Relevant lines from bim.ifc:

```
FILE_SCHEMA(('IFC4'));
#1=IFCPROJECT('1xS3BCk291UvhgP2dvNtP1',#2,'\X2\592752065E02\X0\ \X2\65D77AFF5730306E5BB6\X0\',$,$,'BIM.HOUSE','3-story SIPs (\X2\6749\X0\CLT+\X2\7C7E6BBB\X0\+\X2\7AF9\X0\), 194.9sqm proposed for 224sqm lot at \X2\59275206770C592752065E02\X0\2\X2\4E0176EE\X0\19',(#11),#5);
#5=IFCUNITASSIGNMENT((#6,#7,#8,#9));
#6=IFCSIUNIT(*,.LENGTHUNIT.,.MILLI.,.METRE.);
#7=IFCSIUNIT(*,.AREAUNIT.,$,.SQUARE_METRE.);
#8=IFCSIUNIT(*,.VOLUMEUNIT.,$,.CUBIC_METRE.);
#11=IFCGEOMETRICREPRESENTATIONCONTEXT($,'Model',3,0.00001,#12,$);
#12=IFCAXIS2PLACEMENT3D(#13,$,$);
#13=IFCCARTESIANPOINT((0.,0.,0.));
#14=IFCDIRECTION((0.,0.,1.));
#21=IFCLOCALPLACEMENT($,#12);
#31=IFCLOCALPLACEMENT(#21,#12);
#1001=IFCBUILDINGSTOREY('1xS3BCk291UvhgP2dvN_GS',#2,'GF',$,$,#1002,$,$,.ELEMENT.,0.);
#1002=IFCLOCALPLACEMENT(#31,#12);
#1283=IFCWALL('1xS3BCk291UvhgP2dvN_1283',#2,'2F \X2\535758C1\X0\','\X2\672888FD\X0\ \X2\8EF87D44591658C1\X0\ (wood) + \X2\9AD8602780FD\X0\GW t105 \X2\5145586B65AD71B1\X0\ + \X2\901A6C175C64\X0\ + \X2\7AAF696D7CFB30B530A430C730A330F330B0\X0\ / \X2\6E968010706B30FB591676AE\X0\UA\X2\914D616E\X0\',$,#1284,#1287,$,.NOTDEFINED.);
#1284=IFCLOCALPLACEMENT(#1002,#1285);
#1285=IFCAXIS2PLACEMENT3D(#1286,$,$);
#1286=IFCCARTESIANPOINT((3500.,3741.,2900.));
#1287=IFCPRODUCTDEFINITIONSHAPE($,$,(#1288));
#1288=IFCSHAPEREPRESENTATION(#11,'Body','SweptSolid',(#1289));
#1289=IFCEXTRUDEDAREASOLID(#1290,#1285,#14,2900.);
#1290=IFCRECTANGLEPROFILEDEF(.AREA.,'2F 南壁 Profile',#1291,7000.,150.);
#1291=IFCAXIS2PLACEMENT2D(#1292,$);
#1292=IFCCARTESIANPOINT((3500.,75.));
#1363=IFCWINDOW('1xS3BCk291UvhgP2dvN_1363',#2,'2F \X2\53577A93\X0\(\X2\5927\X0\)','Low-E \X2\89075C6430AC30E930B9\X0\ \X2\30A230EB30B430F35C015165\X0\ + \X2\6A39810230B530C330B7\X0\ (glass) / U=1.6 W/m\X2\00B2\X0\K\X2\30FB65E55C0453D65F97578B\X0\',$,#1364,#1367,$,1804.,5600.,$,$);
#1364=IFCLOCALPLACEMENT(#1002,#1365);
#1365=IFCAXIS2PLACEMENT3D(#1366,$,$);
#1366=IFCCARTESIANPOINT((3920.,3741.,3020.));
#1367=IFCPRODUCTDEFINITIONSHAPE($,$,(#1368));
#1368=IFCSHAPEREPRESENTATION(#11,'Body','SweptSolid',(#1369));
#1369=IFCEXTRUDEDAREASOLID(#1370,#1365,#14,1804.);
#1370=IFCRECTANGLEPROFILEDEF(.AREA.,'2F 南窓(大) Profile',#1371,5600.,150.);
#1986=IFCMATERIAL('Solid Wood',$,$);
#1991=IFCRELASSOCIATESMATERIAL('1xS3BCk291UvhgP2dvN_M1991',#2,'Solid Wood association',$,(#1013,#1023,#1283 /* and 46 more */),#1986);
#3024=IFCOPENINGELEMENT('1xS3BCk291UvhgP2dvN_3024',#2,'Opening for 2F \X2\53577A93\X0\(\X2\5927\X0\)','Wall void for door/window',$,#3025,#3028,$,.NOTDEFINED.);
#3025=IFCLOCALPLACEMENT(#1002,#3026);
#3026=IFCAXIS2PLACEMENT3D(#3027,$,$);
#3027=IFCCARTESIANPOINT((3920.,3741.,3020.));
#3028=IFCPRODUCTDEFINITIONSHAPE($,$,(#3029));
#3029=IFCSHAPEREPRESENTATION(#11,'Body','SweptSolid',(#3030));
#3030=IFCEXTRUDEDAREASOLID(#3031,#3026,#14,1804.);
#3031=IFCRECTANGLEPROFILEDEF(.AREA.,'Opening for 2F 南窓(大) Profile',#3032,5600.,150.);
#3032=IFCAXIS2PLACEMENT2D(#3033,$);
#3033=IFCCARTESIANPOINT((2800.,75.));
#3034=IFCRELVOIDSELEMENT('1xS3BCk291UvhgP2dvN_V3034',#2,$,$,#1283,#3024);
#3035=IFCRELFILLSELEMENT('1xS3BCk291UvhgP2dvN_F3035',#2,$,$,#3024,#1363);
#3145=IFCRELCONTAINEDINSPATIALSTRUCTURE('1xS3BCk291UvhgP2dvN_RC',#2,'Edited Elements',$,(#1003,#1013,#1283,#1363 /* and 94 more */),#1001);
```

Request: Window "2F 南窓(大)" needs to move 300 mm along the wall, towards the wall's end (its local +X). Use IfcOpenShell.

```python
import ifcopenshell
import ifcopenshell.api.geometry
import ifcopenshell.util.placement
import ifcopenshell.util.unit

model = ifcopenshell.open("bim.ifc")
unit_scale = ifcopenshell.util.unit.calculate_unit_scale(model)

window = model.by_guid("1xS3BCk291UvhgP2dvN_1363")
opening = window.FillsVoids[0].RelatingOpeningElement
wall = opening.VoidsElements[0].RelatingBuildingElement

wall_matrix = ifcopenshell.util.placement.get_local_placement(wall.ObjectPlacement)
shift = wall_matrix[:3, 0] * 0.3 / unit_scale
before = ifcopenshell.util.placement.get_local_placement(window.ObjectPlacement)[:3, 3].copy()

# The window is not placed relative to its opening, so move both.
for product in (opening, window):
    matrix = ifcopenshell.util.placement.get_local_placement(product.ObjectPlacement)
    matrix[:3, 3] += shift
    ifcopenshell.api.geometry.edit_object_placement(model, product=product, matrix=matrix, is_si=False)

after = ifcopenshell.util.placement.get_local_placement(window.ObjectPlacement)[:3, 3]
print("window moved by", (after - before).round(3) + 0.0)

model.write("bim_edited.ifc")
```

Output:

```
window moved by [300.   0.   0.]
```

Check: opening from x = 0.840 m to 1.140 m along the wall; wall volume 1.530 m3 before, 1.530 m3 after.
